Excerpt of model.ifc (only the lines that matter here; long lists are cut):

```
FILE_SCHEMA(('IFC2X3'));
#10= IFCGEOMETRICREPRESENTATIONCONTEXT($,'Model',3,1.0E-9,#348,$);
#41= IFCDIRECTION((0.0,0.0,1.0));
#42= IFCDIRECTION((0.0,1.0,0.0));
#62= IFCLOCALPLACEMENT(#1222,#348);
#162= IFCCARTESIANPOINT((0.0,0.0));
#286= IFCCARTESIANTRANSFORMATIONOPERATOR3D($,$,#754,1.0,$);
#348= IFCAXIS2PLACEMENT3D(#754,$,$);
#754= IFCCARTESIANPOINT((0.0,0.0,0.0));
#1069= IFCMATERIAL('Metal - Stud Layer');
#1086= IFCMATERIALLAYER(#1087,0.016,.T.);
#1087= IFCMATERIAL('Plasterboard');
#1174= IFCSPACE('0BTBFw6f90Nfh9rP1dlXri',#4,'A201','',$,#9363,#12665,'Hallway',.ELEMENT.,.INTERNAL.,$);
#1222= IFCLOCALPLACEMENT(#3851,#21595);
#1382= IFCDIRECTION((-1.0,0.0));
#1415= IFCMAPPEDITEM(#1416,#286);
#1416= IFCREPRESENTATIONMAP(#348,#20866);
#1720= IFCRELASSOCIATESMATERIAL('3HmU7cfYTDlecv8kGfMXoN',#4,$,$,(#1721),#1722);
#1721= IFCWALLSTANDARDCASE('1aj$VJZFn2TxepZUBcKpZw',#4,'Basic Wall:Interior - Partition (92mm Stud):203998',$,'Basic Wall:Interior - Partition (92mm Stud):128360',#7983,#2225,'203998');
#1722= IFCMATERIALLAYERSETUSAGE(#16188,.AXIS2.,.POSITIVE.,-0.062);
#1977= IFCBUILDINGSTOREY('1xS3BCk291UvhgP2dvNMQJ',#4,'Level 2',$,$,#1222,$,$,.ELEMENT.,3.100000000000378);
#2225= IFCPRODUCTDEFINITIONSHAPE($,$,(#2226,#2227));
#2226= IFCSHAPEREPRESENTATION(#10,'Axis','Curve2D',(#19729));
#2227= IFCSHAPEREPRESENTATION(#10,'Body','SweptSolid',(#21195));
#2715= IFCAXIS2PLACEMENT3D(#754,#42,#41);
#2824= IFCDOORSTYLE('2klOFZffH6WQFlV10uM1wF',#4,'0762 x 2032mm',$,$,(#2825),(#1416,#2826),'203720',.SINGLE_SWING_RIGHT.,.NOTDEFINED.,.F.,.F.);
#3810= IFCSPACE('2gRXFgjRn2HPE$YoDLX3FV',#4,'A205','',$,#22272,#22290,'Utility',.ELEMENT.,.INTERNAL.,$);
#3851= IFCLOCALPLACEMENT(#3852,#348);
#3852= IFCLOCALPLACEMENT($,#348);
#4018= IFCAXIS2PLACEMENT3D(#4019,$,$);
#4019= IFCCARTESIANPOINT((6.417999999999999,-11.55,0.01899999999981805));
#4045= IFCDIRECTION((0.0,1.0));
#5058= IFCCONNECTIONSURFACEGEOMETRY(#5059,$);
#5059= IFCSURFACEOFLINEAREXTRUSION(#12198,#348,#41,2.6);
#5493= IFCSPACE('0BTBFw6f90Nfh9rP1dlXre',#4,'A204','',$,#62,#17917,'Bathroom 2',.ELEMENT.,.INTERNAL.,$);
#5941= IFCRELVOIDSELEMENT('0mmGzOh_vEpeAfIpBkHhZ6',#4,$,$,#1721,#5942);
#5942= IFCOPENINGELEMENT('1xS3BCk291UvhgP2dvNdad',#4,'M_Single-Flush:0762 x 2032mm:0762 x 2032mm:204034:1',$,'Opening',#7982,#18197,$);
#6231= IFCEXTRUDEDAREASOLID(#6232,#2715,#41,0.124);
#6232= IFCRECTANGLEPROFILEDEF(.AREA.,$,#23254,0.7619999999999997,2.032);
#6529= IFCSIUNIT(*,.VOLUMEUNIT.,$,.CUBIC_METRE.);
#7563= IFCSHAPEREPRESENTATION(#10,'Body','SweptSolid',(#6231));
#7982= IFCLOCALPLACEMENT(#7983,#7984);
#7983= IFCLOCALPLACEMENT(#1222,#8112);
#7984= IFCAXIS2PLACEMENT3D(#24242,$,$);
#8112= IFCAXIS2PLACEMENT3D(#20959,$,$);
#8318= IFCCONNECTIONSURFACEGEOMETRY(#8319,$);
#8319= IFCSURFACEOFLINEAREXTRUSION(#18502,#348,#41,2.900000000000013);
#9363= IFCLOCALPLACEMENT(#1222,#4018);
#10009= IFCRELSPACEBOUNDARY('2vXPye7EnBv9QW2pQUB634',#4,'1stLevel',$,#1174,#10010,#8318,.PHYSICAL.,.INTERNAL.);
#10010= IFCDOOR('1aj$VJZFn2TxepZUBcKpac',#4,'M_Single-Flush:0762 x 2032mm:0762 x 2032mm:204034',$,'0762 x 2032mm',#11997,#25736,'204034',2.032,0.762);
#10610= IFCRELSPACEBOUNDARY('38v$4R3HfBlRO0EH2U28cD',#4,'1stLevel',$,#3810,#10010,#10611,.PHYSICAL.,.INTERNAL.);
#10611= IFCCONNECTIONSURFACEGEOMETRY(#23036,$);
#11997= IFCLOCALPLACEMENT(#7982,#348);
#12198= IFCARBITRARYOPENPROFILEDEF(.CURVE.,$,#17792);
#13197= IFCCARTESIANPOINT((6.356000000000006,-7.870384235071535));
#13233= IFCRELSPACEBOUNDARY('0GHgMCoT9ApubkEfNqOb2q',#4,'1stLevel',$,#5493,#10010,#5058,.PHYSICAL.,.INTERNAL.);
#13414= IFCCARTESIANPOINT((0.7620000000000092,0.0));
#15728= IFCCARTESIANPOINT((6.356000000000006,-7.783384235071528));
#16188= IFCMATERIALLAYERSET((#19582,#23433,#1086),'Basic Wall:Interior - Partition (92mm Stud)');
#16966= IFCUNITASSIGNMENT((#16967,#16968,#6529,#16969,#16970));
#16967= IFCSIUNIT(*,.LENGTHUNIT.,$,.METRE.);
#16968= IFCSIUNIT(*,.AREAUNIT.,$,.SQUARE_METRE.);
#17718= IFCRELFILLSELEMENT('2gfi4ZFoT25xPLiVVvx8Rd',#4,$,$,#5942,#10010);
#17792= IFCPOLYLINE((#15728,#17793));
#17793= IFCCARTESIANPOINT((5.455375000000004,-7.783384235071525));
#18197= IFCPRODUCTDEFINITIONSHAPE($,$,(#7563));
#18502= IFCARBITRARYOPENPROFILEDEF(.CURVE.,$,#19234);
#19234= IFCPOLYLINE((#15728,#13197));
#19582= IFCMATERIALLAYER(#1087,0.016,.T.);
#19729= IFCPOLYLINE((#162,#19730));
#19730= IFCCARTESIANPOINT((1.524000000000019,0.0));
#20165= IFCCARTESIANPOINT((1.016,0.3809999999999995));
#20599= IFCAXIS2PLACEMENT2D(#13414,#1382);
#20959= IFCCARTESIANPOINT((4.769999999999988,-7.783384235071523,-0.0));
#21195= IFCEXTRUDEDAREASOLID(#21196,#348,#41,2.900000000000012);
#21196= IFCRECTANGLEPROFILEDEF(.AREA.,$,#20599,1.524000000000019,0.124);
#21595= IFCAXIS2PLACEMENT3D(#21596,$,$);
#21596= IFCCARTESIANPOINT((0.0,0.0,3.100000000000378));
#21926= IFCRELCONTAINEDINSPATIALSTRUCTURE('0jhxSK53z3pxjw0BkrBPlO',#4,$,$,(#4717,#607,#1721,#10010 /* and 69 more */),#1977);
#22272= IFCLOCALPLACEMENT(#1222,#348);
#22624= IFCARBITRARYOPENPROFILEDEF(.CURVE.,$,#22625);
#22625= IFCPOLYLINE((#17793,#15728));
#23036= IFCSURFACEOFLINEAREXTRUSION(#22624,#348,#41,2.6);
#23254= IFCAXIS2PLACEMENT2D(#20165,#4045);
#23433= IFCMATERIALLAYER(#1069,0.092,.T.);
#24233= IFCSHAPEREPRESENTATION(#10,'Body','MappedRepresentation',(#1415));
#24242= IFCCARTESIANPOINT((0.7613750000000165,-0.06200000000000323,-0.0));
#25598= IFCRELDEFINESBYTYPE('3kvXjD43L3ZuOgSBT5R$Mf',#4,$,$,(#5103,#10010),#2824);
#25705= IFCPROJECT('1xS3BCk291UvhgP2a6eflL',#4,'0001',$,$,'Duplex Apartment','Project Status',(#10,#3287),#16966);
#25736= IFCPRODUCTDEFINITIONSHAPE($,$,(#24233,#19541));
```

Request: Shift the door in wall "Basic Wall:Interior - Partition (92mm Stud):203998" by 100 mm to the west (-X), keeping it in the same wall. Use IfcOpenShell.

```python
import numpy as np
import ifcopenshell
import ifcopenshell.api.geometry
import ifcopenshell.util.placement
import ifcopenshell.util.unit

model = ifcopenshell.open("model.ifc")
unit_scale = ifcopenshell.util.unit.calculate_unit_scale(model)

door = model.by_guid("1aj$VJZFn2TxepZUBcKpac")
opening = door.FillsVoids[0].RelatingOpeningElement
wall = opening.VoidsElements[0].RelatingBuildingElement

wall_matrix = ifcopenshell.util.placement.get_local_placement(wall.ObjectPlacement)
shift = wall_matrix[:3, 0] * -0.1 / unit_scale
before = ifcopenshell.util.placement.get_local_placement(door.ObjectPlacement)[:3, 3].copy()

# The door is placed relative to its opening, so it follows when the opening moves.
matrix = ifcopenshell.util.placement.get_local_placement(opening.ObjectPlacement)
matrix[:3, 3] += shift
ifcopenshell.api.geometry.edit_object_placement(
    model, product=opening, matrix=matrix, is_si=False, should_transform_children=True
)

# Space boundary surfaces are stored in each space's coordinates; move them too.
for rel in door.ProvidesBoundaries:
    if not rel.ConnectionGeometry:
        continue
    surface = rel.ConnectionGeometry.SurfaceOnRelatingElement
    space_matrix = ifcopenshell.util.placement.get_local_placement(rel.RelatingSpace.ObjectPlacement)
    point = np.array(surface.Position.Location.Coordinates) + space_matrix[:3, :3].T @ shift
    surface.Position = model.createIfcAxis2Placement3D(
        model.createIfcCartesianPoint(point.tolist()), surface.Position.Axis, surface.Position.RefDirection
    )

after = ifcopenshell.util.placement.get_local_placement(door.ObjectPlacement)[:3, 3]
print("door moved by", (after - before).round(3) + 0.0)

model.write("model_rev.ifc")
```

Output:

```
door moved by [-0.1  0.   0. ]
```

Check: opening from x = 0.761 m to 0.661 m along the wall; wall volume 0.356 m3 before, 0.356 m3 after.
